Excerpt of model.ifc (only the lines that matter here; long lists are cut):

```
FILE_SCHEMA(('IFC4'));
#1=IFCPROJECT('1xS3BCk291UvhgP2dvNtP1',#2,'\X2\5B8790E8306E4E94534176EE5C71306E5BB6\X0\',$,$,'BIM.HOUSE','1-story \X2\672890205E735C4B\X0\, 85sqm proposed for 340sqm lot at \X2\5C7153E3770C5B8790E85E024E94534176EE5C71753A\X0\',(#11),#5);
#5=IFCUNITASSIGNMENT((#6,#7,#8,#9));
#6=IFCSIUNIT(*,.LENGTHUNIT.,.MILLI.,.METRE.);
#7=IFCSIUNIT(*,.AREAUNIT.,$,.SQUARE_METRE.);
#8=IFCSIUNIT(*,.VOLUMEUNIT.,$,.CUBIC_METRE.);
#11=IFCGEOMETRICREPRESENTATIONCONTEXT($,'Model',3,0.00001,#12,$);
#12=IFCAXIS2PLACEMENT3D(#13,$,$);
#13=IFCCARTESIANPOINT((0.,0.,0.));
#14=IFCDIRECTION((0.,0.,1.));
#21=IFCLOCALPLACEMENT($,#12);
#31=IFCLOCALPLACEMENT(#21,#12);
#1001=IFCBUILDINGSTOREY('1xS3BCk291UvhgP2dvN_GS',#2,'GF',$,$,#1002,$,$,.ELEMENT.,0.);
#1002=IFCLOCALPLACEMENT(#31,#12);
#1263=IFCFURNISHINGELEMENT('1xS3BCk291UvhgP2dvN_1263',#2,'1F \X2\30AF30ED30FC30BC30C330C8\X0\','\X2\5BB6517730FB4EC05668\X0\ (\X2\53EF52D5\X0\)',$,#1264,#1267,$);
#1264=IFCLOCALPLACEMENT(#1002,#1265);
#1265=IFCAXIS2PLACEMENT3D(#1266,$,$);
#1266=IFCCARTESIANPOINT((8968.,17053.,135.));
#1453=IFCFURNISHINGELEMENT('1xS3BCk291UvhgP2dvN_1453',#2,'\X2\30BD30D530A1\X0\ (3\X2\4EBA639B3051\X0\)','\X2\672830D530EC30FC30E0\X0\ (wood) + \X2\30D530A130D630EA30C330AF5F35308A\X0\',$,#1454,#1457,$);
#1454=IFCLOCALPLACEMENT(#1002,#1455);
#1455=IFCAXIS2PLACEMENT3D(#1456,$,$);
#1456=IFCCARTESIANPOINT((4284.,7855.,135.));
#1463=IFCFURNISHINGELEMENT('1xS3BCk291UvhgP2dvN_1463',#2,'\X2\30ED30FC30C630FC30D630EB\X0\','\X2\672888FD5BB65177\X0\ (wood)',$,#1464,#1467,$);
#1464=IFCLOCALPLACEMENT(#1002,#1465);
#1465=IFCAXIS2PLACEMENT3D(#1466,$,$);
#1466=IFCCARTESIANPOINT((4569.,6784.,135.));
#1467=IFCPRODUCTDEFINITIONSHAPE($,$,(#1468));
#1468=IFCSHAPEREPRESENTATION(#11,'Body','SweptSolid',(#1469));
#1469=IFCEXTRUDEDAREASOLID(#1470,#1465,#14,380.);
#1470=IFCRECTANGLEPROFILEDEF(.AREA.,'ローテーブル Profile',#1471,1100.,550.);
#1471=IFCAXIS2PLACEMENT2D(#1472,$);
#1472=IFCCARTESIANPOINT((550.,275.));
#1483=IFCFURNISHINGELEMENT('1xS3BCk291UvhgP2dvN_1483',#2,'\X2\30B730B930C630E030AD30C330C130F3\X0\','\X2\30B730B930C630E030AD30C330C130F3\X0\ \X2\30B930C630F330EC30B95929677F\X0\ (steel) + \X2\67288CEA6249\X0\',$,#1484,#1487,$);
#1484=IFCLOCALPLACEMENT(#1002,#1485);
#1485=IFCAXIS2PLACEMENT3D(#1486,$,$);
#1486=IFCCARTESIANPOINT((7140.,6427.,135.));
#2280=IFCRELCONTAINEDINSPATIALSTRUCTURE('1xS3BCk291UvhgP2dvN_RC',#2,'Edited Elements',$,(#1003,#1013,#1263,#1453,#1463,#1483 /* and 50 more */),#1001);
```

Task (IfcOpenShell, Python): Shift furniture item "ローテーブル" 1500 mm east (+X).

```python
import ifcopenshell
import ifcopenshell.api.geometry
import ifcopenshell.util.placement
import ifcopenshell.util.unit

model = ifcopenshell.open("model.ifc")
unit_scale = ifcopenshell.util.unit.calculate_unit_scale(model)

item = model.by_guid("1xS3BCk291UvhgP2dvN_1463")
matrix = ifcopenshell.util.placement.get_local_placement(item.ObjectPlacement)
matrix[0, 3] += 1.5 / unit_scale
ifcopenshell.api.geometry.edit_object_placement(model, product=item, matrix=matrix, is_si=False)

print(ifcopenshell.util.placement.get_local_placement(item.ObjectPlacement).round(3) + 0.0)

model.write("model_rev.ifc")
```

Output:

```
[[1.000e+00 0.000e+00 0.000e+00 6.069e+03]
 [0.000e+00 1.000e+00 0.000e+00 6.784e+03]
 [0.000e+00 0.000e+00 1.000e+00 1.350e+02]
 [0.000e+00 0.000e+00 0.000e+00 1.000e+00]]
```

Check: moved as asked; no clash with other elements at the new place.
